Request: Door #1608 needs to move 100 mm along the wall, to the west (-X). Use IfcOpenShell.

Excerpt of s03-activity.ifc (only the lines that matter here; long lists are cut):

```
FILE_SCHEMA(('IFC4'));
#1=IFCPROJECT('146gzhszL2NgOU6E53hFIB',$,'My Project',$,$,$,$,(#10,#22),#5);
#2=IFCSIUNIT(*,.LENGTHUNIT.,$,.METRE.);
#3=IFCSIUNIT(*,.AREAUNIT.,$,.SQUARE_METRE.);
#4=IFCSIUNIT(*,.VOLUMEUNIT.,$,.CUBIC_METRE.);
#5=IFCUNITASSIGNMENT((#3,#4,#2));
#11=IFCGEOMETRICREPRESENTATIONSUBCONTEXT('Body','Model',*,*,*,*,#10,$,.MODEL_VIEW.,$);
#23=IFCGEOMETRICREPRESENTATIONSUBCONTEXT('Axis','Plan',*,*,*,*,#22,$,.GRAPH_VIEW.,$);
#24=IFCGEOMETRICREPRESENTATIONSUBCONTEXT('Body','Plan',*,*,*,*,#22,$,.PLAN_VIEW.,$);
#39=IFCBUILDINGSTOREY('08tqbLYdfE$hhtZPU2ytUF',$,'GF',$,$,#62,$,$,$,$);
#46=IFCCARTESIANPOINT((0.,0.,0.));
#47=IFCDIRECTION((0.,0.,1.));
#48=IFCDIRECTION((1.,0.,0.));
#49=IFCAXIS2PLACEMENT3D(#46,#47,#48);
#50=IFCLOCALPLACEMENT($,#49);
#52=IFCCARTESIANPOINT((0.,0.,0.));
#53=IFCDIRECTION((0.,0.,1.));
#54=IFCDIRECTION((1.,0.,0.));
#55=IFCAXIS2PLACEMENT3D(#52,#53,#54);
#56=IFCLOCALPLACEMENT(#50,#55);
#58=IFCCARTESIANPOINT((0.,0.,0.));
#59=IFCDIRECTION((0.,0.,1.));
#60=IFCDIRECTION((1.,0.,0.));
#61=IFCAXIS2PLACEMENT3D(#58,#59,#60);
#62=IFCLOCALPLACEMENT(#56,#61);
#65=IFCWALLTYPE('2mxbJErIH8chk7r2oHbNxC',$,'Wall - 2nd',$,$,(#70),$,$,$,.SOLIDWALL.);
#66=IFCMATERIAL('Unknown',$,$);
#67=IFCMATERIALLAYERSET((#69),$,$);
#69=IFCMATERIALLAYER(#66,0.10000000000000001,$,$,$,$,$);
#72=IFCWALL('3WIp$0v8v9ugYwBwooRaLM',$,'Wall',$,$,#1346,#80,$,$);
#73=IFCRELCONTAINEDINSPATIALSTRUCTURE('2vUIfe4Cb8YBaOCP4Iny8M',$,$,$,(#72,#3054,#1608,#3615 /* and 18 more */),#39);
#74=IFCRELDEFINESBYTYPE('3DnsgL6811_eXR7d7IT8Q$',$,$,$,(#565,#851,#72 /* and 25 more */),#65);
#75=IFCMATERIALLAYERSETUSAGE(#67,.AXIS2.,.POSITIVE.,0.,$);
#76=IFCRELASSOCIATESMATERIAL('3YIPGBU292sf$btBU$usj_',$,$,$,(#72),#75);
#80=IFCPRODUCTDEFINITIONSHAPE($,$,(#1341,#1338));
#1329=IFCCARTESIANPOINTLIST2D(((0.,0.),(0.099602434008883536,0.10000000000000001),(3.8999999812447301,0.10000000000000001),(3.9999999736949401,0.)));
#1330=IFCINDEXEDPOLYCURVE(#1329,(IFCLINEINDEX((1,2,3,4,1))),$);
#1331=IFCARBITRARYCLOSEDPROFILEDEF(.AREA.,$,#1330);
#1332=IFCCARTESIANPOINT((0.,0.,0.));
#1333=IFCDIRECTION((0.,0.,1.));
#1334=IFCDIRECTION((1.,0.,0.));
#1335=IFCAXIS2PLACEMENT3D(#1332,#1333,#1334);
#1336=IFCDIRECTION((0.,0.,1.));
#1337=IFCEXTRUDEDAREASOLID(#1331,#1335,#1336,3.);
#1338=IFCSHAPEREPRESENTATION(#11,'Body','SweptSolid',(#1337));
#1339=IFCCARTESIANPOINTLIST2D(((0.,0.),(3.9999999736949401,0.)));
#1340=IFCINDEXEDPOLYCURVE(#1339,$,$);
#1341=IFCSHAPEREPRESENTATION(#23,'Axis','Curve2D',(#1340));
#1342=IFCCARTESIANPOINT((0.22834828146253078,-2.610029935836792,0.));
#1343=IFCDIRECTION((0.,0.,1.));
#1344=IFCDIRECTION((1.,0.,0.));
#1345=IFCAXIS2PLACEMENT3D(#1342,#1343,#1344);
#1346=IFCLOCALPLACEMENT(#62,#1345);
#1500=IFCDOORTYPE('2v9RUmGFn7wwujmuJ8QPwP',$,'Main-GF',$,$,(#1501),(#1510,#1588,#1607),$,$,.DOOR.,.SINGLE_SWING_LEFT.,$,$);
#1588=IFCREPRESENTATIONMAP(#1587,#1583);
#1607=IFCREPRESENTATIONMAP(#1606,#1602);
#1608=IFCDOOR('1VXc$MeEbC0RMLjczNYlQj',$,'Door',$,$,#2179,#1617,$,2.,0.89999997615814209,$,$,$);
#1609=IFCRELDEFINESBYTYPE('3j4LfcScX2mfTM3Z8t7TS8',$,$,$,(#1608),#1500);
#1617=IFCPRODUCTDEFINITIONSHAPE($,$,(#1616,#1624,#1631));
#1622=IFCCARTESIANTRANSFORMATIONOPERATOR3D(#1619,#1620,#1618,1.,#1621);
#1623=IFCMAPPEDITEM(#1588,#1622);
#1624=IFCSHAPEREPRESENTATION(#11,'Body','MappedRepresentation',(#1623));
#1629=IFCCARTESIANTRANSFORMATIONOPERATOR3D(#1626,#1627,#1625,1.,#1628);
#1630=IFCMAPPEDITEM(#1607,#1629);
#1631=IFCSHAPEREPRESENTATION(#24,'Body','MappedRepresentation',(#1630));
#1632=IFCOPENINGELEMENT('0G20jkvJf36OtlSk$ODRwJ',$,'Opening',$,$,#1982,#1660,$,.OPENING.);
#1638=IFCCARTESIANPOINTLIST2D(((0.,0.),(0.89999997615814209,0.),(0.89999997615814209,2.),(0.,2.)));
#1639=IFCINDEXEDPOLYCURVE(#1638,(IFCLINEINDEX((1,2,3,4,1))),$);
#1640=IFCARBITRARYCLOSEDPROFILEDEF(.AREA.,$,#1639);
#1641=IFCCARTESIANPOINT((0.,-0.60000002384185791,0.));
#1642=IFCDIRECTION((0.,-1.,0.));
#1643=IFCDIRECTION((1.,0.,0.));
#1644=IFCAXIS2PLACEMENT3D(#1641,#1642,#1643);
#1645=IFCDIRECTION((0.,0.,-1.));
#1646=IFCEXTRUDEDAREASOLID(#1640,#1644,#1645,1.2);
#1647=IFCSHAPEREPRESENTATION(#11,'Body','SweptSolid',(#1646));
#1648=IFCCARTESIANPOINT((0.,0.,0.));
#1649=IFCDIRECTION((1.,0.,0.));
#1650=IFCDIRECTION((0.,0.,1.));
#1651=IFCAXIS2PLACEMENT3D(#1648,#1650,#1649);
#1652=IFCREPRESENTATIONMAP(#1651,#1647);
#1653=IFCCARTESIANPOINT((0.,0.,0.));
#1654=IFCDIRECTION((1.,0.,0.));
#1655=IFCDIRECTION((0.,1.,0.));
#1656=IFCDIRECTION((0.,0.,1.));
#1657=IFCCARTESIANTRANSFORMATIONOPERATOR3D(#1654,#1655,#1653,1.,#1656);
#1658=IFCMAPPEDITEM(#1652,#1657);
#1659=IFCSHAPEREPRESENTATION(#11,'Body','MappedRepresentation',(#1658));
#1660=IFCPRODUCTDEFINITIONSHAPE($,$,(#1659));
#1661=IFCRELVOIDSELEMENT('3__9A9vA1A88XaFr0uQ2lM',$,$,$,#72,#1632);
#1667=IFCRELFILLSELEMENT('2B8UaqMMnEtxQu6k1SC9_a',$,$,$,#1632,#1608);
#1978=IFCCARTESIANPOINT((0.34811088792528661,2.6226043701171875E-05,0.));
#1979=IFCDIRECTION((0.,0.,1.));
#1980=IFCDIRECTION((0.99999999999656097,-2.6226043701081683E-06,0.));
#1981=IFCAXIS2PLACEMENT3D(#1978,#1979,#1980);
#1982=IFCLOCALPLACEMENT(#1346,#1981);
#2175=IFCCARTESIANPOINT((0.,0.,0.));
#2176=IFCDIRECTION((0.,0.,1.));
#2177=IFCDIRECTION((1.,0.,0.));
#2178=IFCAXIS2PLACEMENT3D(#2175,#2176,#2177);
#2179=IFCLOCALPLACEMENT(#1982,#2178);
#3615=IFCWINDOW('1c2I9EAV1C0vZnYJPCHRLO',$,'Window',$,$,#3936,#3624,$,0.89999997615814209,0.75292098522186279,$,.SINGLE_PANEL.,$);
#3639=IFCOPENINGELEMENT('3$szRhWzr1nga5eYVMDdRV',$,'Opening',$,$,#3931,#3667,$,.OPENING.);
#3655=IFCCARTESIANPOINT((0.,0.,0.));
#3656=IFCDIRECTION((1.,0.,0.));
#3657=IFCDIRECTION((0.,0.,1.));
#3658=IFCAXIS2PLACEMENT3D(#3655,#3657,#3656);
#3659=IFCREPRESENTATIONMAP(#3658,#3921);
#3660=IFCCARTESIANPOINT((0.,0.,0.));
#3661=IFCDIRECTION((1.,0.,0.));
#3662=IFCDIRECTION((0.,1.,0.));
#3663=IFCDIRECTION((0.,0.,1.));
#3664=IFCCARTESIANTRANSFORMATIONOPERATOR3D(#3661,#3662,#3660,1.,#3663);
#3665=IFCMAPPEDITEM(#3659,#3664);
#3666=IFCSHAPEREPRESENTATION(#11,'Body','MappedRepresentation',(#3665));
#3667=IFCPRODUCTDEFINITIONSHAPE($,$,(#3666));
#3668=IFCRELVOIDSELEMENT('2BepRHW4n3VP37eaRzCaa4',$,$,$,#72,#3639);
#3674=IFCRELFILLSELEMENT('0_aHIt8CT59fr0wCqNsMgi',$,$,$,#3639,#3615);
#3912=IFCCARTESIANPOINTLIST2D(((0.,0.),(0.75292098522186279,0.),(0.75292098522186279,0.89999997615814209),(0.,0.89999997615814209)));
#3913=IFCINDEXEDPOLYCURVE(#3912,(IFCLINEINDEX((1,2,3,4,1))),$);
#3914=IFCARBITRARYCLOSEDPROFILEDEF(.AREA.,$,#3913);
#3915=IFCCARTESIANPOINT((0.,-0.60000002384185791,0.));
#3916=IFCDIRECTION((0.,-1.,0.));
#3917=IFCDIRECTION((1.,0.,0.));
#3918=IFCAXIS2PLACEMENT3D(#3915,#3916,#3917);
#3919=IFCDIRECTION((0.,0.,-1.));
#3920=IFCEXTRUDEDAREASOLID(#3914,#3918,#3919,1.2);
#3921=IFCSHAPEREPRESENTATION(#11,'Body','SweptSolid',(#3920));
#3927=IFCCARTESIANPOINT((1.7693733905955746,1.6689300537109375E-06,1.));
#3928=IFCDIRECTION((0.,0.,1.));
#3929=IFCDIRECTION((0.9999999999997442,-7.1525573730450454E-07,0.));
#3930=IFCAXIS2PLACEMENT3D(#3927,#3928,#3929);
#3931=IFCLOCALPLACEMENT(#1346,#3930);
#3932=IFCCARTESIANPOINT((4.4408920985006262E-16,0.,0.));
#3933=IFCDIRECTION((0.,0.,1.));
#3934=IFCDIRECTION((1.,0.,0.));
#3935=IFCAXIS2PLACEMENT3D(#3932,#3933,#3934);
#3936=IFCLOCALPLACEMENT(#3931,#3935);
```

```python
import ifcopenshell
import ifcopenshell.api.geometry
import ifcopenshell.util.placement
import ifcopenshell.util.unit

model = ifcopenshell.open("s03-activity.ifc")
unit_scale = ifcopenshell.util.unit.calculate_unit_scale(model)

door = model.by_guid("1VXc$MeEbC0RMLjczNYlQj")
opening = door.FillsVoids[0].RelatingOpeningElement
wall = opening.VoidsElements[0].RelatingBuildingElement

wall_matrix = ifcopenshell.util.placement.get_local_placement(wall.ObjectPlacement)
shift = wall_matrix[:3, 0] * -0.1 / unit_scale
before = ifcopenshell.util.placement.get_local_placement(door.ObjectPlacement)[:3, 3].copy()

# The door is placed relative to its opening, so it follows when the opening moves.
matrix = ifcopenshell.util.placement.get_local_placement(opening.ObjectPlacement)
matrix[:3, 3] += shift
ifcopenshell.api.geometry.edit_object_placement(
    model, product=opening, matrix=matrix, is_si=False, should_transform_children=True
)

after = ifcopenshell.util.placement.get_local_placement(door.ObjectPlacement)[:3, 3]
print("door moved by", (after - before).round(3) + 0.0)

model.write("s03-activity-out.ifc")
```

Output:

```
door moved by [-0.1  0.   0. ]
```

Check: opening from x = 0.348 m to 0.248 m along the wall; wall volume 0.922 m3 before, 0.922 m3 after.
